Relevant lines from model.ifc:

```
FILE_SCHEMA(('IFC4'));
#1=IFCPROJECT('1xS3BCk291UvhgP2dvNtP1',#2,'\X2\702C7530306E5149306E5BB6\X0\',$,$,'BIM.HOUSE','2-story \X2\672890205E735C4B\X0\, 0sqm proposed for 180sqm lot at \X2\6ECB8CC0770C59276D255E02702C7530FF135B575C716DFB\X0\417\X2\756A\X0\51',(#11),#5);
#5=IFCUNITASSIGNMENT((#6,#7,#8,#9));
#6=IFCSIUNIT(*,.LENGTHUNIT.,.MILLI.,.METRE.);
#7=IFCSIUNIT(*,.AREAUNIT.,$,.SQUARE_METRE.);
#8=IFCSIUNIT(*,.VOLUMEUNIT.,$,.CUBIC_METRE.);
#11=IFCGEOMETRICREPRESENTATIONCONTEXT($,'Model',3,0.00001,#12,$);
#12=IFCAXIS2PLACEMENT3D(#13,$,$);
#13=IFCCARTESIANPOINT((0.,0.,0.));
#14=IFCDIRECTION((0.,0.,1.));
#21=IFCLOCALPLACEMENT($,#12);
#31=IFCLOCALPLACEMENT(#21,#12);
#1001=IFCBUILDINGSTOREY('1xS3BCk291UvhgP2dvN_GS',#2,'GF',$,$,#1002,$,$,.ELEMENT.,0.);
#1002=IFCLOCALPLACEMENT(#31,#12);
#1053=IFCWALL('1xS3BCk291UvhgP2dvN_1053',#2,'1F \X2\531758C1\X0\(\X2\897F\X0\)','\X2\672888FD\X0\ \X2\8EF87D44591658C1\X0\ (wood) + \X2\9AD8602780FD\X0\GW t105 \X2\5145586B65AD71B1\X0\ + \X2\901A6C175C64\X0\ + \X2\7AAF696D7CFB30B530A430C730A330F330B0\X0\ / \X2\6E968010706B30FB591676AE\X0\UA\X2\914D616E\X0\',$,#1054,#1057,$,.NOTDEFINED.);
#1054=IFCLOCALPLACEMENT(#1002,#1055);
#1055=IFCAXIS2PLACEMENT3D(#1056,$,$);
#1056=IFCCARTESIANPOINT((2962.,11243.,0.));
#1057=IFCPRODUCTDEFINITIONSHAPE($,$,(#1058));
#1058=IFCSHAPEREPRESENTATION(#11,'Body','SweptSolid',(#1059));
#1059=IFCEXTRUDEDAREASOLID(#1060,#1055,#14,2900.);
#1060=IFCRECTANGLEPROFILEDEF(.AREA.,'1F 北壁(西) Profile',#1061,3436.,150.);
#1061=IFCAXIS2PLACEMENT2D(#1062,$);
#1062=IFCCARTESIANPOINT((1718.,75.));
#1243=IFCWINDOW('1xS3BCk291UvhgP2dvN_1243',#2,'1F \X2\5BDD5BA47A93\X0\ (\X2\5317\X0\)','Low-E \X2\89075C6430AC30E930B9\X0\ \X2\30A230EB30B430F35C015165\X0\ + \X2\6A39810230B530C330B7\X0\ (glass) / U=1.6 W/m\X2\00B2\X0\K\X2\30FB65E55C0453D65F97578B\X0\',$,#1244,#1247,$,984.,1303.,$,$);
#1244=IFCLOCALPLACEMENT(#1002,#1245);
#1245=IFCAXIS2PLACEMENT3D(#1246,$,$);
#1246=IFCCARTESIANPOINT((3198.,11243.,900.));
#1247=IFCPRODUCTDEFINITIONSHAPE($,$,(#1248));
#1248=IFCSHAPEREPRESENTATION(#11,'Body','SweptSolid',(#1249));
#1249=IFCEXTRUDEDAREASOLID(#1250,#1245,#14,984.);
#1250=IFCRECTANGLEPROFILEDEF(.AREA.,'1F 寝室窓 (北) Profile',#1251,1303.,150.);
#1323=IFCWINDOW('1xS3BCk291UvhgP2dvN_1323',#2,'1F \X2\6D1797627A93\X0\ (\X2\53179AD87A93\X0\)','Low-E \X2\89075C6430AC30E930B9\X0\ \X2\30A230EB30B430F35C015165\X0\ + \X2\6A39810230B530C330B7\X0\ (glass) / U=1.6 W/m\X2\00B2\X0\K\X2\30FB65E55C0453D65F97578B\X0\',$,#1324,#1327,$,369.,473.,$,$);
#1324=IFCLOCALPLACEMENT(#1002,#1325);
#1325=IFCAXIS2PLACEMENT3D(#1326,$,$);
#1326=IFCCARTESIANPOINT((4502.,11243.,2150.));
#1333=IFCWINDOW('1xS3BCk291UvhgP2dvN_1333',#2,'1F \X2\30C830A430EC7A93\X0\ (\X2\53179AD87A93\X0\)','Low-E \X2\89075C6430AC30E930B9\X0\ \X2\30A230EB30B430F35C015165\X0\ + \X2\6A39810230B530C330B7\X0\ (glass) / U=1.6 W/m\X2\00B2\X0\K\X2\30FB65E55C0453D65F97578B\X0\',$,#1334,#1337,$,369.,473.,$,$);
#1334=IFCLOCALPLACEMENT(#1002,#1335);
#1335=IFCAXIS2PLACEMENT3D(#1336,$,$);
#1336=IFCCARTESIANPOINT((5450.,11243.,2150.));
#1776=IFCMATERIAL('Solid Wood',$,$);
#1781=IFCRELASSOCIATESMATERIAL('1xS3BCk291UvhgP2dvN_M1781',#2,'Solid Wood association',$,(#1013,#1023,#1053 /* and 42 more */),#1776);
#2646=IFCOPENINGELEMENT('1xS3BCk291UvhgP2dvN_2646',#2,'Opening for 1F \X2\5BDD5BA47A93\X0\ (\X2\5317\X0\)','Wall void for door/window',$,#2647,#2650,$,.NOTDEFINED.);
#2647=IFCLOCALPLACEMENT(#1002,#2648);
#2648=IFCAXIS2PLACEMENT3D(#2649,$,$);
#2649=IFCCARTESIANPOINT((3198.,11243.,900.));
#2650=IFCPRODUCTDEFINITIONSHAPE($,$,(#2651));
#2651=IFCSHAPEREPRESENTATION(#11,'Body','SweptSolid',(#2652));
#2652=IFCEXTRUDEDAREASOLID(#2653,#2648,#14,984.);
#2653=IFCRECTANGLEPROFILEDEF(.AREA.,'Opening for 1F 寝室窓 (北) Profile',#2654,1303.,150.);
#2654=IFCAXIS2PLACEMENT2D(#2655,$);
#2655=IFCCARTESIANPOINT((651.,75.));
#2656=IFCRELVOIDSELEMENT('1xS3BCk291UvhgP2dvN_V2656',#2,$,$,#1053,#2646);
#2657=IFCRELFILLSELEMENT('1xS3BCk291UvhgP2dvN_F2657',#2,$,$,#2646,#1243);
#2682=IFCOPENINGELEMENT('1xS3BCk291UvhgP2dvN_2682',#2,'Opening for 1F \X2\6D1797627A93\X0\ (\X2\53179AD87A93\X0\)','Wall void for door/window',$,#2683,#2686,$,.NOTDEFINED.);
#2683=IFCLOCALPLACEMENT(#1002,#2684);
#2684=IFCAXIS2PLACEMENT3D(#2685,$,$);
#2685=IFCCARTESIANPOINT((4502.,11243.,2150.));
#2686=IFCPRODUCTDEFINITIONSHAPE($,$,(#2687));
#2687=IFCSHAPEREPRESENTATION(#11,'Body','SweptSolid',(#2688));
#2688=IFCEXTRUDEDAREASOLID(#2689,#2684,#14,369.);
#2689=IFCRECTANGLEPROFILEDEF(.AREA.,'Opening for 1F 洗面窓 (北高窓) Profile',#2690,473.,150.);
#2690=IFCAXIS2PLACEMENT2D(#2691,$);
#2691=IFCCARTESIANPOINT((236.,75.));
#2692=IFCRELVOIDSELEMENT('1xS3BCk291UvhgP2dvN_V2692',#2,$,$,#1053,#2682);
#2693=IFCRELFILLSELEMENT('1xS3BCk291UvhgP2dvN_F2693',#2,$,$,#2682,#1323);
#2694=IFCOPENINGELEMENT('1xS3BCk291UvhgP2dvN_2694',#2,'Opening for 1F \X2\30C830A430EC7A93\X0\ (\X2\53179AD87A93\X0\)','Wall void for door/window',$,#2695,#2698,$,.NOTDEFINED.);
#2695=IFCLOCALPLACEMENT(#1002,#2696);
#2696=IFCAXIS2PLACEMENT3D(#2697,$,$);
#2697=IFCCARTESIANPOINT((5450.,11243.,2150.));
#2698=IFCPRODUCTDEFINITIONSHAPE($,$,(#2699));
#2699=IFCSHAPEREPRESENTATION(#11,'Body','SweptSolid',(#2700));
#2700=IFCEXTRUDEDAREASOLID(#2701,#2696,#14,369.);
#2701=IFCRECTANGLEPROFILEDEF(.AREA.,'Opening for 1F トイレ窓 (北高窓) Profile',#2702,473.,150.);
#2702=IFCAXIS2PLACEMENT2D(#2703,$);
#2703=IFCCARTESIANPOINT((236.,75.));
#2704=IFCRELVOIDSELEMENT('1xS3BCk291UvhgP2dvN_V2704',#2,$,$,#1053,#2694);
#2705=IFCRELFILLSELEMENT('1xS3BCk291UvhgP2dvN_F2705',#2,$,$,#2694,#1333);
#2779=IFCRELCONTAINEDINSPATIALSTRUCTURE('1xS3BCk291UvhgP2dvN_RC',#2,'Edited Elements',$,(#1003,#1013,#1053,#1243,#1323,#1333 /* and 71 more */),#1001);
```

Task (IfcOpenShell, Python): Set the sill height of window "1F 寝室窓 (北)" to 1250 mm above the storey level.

```python
import numpy as np
import ifcopenshell
import ifcopenshell.api.geometry
import ifcopenshell.geom
import ifcopenshell.util.element
import ifcopenshell.util.placement
import ifcopenshell.util.shape
import ifcopenshell.util.unit

model = ifcopenshell.open("model.ifc")
unit_scale = ifcopenshell.util.unit.calculate_unit_scale(model)

window = model.by_id(1243)
opening = window.FillsVoids[0].RelatingOpeningElement
storey = ifcopenshell.util.element.get_container(window, ifc_class="IfcBuildingStorey")
level = ifcopenshell.util.placement.get_local_placement(storey.ObjectPlacement)[2, 3]

# The opening's origin need not be at the sill, so measure its lowest point.
shape = ifcopenshell.geom.create_shape(ifcopenshell.geom.settings(), opening)
bottom = ifcopenshell.util.shape.get_shape_bottom_elevation(shape, shape.geometry) / unit_scale
dz = level + 1250.0 - bottom

shift = np.array([0.0, 0.0, dz])
# The window is not placed relative to its opening, so move both.
for product in (opening, window):
    matrix = ifcopenshell.util.placement.get_local_placement(product.ObjectPlacement)
    matrix[:3, 3] += shift
    ifcopenshell.api.geometry.edit_object_placement(model, product=product, matrix=matrix, is_si=False)

print(f"moved by {dz * unit_scale:+.3f} m")

model.write("model-out.ifc")
```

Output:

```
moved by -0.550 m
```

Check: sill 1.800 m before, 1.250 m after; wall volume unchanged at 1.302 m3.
